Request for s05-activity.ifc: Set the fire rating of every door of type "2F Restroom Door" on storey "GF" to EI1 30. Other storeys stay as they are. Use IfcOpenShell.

First a look at what the model holds.

```python
import ifcopenshell
import ifcopenshell.util.element

model = ifcopenshell.open("s05-activity.ifc")
print(model.schema)
storey = next(s for s in model.by_type("IfcBuildingStorey") if s.Name == "GF")
doors = [e for e in ifcopenshell.util.element.get_decomposition(storey) if e.is_a("IfcDoor")]
seen = {}
for e in doors:
    element_type = ifcopenshell.util.element.get_type(e)
    key = (element_type.Name if element_type != e and element_type else None, ifcopenshell.util.element.get_pset(e, "Pset_DoorCommon", "FireRating"))
    seen[key] = seen.get(key, 0) + 1
for (name, value), count in sorted(seen.items(), key=str):
    print(count, "x", name, "|", value)
```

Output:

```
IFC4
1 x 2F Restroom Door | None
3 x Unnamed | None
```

```python
import ifcopenshell
import ifcopenshell.api.pset
import ifcopenshell.util.element

model = ifcopenshell.open("s05-activity.ifc")

storey = next(s for s in model.by_type("IfcBuildingStorey") if s.Name == "GF")
doors = [e for e in ifcopenshell.util.element.get_decomposition(storey) if e.is_a("IfcDoor")]

count = 0
for e in doors:
    element_type = ifcopenshell.util.element.get_type(e)
    if element_type in (None, e) or element_type.Name != "2F Restroom Door":
        continue
    # add_pset returns the element's existing set when there is one.
    pset = ifcopenshell.api.pset.add_pset(model, product=e, name="Pset_DoorCommon")
    ifcopenshell.api.pset.edit_pset(model, pset=pset, properties={"FireRating": "EI1 30"})
    count += 1

print(count, "doors updated")

model.write("s05-activity_rev.ifc")
```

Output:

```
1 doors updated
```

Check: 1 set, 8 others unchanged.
